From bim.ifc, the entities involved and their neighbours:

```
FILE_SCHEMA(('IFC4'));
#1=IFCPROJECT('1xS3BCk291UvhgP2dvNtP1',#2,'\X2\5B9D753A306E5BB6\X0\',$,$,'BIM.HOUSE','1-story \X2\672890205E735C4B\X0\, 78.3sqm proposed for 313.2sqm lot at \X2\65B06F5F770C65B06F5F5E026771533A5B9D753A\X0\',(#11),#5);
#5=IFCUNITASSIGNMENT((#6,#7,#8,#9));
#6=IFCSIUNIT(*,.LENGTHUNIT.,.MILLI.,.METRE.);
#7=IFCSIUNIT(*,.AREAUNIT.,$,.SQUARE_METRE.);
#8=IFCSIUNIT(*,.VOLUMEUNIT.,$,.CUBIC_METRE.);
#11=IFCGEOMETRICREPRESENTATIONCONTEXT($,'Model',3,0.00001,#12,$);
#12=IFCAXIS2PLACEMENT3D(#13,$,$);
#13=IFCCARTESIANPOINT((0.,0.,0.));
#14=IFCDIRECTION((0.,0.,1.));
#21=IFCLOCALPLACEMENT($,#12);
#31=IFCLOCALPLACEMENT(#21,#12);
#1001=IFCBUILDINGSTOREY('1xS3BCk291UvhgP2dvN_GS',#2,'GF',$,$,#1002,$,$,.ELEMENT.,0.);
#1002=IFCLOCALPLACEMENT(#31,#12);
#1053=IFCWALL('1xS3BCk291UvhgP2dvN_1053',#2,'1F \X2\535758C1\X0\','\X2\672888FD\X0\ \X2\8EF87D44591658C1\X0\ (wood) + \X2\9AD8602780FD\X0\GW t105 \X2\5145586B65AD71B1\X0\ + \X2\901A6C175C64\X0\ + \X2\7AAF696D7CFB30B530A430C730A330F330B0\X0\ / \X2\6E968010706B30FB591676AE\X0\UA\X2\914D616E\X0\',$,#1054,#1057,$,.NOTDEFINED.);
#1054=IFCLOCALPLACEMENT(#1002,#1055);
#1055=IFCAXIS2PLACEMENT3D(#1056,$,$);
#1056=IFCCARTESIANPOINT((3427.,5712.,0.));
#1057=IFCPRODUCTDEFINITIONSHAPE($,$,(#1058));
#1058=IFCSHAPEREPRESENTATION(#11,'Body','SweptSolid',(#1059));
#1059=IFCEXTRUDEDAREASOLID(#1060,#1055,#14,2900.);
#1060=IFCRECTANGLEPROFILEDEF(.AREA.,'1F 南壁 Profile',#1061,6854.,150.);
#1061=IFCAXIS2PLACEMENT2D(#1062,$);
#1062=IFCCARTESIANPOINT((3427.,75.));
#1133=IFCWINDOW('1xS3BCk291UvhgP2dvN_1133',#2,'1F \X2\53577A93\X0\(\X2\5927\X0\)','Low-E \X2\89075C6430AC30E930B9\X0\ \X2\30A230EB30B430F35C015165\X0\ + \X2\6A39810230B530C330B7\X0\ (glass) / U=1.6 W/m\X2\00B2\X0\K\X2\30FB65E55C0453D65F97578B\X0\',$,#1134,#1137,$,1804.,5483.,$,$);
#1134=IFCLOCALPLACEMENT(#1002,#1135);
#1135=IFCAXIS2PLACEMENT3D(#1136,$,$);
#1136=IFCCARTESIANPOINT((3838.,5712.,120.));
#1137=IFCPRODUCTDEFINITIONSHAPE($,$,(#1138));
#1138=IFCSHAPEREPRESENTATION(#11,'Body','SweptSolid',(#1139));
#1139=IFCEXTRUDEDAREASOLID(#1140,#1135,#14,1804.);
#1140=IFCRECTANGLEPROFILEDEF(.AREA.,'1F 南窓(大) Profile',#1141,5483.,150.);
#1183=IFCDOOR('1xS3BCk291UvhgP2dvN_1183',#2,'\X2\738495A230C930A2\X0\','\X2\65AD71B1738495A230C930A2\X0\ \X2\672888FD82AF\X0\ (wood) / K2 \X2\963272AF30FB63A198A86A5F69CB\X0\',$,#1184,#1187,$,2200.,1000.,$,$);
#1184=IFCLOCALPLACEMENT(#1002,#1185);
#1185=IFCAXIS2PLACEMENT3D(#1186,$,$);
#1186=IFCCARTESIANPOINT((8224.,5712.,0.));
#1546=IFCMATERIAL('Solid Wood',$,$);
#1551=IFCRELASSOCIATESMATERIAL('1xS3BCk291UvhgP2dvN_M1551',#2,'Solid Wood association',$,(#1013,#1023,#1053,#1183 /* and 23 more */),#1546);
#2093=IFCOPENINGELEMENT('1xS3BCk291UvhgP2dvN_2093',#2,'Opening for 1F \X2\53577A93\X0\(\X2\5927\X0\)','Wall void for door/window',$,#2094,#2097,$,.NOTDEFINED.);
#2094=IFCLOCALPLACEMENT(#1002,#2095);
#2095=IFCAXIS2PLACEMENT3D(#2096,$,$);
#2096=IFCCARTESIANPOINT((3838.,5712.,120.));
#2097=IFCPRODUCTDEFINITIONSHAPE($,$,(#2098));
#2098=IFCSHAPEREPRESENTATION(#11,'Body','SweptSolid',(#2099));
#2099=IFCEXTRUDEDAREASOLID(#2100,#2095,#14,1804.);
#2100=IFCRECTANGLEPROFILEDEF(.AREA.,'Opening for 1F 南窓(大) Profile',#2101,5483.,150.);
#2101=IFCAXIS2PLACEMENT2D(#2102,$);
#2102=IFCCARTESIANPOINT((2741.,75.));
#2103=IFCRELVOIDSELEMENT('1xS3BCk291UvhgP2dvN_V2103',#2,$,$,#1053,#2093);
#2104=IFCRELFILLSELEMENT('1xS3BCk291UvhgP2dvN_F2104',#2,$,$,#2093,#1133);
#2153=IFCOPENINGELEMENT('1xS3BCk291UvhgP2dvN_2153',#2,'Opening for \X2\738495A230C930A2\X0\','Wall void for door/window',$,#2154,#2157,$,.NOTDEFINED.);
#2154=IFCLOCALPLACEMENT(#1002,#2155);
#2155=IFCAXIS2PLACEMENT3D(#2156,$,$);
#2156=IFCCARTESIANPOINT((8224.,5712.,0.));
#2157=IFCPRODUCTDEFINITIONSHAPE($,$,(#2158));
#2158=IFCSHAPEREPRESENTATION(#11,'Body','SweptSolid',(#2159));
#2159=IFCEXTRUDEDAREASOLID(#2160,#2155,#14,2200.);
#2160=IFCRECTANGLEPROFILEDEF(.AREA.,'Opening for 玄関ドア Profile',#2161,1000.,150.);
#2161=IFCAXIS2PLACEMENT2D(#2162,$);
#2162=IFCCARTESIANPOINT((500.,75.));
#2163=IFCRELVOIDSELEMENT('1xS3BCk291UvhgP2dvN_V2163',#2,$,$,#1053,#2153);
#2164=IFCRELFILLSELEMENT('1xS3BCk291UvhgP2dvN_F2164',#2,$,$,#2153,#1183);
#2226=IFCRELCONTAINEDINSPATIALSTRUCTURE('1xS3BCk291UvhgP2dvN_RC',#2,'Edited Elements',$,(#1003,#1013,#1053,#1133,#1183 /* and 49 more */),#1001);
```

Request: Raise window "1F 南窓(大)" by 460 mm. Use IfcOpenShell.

```python
import numpy as np
import ifcopenshell
import ifcopenshell.api.geometry
import ifcopenshell.util.placement
import ifcopenshell.util.unit

model = ifcopenshell.open("bim.ifc")
unit_scale = ifcopenshell.util.unit.calculate_unit_scale(model)

window = model.by_id(1133)
opening = window.FillsVoids[0].RelatingOpeningElement
dz = 0.46 / unit_scale

shift = np.array([0.0, 0.0, dz])
# The window is not placed relative to its opening, so move both.
for product in (opening, window):
    matrix = ifcopenshell.util.placement.get_local_placement(product.ObjectPlacement)
    matrix[:3, 3] += shift
    ifcopenshell.api.geometry.edit_object_placement(model, product=product, matrix=matrix, is_si=False)

print(f"moved by {dz * unit_scale:+.3f} m")

model.write("bim_edited.ifc")
```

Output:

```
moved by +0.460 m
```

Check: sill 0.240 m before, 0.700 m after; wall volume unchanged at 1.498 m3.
